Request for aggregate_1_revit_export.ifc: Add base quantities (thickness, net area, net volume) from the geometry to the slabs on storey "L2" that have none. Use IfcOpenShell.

First a look at what the model holds.

```python
import ifcopenshell
import ifcopenshell.util.element
import ifcopenshell.util.unit

model = ifcopenshell.open("aggregate_1_revit_export.ifc")
print(model.schema)
for unit_type in ("LENGTHUNIT", "AREAUNIT", "VOLUMEUNIT"):
    print(unit_type, ifcopenshell.util.unit.calculate_unit_scale(model, unit_type))
storey = next(s for s in model.by_type("IfcBuildingStorey") if s.Name == "L2")
slabs = [e for e in ifcopenshell.util.element.get_decomposition(storey) if e.is_a("IfcSlab")]
for e in sorted(slabs, key=lambda e: e.id()):
    print(e.id(), e.is_a(), e.Name, list(ifcopenshell.util.element.get_psets(e, qtos_only=True)), sep=" | ")
```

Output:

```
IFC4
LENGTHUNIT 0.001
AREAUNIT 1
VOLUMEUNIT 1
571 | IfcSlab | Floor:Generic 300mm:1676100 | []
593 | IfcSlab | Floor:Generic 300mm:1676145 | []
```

```python
import ifcopenshell
import ifcopenshell.api.pset
import ifcopenshell.geom
import ifcopenshell.util.element
import ifcopenshell.util.shape
import ifcopenshell.util.unit

model = ifcopenshell.open("aggregate_1_revit_export.ifc")
unit_scale = ifcopenshell.util.unit.calculate_unit_scale(model)
area_scale = ifcopenshell.util.unit.calculate_unit_scale(model, "AREAUNIT")
volume_scale = ifcopenshell.util.unit.calculate_unit_scale(model, "VOLUMEUNIT")
settings = ifcopenshell.geom.settings()

storey = next(s for s in model.by_type("IfcBuildingStorey") if s.Name == "L2")
slabs = [e for e in ifcopenshell.util.element.get_decomposition(storey) if e.is_a("IfcSlab")]

for e in sorted(slabs, key=lambda e: e.id()):
    if ifcopenshell.util.element.get_psets(e, qtos_only=True, should_inherit=False):
        continue
    # Geometry comes back in metres, in the element's own axes.
    shape = ifcopenshell.geom.create_shape(settings, e)
    values = {
        "Width": ifcopenshell.util.shape.get_z(shape.geometry) / unit_scale,
        "NetArea": ifcopenshell.util.shape.get_footprint_area(shape.geometry) / area_scale,
        "NetVolume": ifcopenshell.util.shape.get_volume(shape.geometry) / volume_scale,
    }
    qto = ifcopenshell.api.pset.add_qto(model, product=e, name="Qto_SlabBaseQuantities")
    ifcopenshell.api.pset.edit_qto(model, qto=qto, properties=values)
    print(e.id(), {k: round(v, 3) for k, v in values.items()})

model.write("aggregate_1_revit_export_updated.ifc")
```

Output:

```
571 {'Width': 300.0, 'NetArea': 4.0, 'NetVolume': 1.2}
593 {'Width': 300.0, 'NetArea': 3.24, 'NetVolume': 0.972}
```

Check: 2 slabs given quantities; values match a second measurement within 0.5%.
